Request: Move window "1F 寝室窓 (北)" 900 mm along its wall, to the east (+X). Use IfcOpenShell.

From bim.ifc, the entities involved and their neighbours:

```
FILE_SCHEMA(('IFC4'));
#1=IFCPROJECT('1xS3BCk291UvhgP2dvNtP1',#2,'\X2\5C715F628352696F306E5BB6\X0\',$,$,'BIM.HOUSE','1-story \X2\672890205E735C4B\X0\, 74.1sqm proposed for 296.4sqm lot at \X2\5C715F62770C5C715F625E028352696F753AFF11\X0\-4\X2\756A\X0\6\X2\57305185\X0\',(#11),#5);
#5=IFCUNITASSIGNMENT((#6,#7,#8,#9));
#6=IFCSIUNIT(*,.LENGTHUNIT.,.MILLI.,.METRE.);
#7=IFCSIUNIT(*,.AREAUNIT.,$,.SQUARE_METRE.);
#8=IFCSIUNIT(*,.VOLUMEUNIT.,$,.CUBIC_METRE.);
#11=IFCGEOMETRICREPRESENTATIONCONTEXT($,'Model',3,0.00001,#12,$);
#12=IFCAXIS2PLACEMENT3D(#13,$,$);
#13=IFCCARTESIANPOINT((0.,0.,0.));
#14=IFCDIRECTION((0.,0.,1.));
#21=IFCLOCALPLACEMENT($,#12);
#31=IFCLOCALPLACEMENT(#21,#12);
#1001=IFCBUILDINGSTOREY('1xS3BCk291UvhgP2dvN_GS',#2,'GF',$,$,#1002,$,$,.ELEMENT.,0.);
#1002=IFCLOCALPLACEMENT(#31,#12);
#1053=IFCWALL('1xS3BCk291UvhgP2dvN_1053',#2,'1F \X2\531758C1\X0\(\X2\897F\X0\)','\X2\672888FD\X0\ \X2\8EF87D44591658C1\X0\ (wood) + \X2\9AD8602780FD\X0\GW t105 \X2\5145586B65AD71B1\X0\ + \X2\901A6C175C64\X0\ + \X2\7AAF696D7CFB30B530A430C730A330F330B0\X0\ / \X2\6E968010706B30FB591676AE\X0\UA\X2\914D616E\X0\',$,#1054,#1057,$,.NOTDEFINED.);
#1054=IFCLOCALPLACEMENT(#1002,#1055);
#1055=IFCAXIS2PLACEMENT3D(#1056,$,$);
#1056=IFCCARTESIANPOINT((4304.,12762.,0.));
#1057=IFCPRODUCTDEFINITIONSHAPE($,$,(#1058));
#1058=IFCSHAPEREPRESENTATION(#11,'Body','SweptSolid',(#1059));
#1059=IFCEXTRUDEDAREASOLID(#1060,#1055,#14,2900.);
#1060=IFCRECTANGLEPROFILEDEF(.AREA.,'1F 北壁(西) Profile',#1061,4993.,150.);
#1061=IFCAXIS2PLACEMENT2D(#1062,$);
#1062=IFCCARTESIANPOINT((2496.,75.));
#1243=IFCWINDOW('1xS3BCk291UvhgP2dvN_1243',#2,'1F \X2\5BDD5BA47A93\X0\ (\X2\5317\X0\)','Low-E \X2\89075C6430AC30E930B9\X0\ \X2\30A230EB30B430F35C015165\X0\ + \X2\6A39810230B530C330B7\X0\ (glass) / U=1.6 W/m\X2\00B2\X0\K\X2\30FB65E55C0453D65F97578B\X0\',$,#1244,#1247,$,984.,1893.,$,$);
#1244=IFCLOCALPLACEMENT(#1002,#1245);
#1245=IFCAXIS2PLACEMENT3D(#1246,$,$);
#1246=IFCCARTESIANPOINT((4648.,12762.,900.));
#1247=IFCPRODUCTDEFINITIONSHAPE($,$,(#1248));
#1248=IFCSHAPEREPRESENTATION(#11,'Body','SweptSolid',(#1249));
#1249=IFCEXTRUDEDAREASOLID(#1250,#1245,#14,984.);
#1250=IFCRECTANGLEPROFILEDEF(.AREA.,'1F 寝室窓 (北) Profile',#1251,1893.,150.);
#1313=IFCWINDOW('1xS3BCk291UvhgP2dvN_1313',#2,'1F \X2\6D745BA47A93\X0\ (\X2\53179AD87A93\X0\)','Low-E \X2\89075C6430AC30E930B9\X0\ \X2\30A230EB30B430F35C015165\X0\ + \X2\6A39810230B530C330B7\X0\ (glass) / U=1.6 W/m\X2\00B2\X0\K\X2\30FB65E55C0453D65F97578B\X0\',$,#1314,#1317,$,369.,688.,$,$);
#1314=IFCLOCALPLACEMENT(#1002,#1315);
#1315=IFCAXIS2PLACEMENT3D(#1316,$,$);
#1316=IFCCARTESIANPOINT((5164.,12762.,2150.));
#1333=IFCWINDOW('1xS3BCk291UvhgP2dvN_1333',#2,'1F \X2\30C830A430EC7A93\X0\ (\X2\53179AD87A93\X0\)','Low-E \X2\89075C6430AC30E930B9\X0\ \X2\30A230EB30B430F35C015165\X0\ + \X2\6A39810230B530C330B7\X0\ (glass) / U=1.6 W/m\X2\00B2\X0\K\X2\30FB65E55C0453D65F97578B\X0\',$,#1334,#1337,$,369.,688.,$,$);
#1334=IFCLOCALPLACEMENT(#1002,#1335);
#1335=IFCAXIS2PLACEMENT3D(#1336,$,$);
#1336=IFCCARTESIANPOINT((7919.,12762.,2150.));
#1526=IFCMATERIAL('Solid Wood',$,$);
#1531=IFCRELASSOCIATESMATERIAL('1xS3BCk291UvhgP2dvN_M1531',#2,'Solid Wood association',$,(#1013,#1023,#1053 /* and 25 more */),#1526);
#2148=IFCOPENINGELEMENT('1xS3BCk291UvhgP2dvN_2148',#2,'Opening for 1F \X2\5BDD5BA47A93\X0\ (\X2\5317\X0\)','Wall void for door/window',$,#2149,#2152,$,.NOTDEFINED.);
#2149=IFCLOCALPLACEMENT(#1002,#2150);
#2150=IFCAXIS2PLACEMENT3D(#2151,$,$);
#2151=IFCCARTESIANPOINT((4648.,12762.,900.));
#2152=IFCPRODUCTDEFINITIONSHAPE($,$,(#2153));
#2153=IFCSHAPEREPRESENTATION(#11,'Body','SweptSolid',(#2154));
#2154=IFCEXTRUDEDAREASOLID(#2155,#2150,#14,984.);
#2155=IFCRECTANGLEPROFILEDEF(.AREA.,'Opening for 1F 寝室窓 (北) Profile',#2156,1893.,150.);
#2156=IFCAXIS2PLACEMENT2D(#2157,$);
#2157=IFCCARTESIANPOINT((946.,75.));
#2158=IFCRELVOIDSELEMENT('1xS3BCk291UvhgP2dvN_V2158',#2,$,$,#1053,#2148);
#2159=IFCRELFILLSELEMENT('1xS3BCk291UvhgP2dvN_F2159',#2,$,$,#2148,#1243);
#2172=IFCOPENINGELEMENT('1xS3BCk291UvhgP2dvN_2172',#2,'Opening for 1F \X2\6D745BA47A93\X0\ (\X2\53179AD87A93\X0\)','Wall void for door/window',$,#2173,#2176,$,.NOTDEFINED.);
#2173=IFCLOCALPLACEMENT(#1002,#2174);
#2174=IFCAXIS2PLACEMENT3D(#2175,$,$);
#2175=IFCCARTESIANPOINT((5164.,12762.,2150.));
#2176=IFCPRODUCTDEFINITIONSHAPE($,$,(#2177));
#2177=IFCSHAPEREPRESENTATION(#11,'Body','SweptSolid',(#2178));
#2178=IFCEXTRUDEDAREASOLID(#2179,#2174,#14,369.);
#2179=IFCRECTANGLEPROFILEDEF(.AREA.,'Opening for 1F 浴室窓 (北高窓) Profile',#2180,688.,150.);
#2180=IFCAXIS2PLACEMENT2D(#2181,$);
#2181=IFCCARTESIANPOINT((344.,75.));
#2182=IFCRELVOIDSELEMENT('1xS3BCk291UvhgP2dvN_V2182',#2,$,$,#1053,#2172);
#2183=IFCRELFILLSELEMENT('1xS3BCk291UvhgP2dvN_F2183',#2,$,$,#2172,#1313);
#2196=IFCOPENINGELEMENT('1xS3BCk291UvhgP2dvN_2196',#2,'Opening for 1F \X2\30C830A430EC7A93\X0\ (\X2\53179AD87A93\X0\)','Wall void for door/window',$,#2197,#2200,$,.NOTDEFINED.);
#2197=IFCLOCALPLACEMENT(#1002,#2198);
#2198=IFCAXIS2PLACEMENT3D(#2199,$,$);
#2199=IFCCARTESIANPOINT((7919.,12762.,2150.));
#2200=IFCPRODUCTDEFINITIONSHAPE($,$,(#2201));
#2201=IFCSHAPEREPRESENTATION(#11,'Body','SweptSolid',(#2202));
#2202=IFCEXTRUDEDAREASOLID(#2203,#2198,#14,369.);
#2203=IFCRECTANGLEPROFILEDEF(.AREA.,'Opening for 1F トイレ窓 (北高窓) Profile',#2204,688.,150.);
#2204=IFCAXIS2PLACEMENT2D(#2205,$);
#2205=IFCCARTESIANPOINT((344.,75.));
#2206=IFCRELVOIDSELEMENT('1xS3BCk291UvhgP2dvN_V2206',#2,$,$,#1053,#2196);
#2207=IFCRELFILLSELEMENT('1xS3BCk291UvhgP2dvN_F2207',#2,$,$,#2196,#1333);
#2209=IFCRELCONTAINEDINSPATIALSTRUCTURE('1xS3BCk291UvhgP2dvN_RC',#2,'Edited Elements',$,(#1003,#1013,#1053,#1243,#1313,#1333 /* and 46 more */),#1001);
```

```python
import ifcopenshell
import ifcopenshell.api.geometry
import ifcopenshell.util.placement

model = ifcopenshell.open("bim.ifc")

window = model.by_guid("1xS3BCk291UvhgP2dvN_1243")
opening = window.FillsVoids[0].RelatingOpeningElement
wall = opening.VoidsElements[0].RelatingBuildingElement

wall_matrix = ifcopenshell.util.placement.get_local_placement(wall.ObjectPlacement)
shift = wall_matrix[:3, 0] * 900.0
before = ifcopenshell.util.placement.get_local_placement(window.ObjectPlacement)[:3, 3].copy()

# The window is not placed relative to its opening, so move both.
for product in (opening, window):
    matrix = ifcopenshell.util.placement.get_local_placement(product.ObjectPlacement)
    matrix[:3, 3] += shift
    ifcopenshell.api.geometry.edit_object_placement(model, product=product, matrix=matrix, is_si=False)

after = ifcopenshell.util.placement.get_local_placement(window.ObjectPlacement)[:3, 3]
print("window moved by", (after - before).round(3) + 0.0)

model.write("bim_updated.ifc")
```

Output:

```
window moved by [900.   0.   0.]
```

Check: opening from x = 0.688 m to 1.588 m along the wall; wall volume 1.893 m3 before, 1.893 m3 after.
